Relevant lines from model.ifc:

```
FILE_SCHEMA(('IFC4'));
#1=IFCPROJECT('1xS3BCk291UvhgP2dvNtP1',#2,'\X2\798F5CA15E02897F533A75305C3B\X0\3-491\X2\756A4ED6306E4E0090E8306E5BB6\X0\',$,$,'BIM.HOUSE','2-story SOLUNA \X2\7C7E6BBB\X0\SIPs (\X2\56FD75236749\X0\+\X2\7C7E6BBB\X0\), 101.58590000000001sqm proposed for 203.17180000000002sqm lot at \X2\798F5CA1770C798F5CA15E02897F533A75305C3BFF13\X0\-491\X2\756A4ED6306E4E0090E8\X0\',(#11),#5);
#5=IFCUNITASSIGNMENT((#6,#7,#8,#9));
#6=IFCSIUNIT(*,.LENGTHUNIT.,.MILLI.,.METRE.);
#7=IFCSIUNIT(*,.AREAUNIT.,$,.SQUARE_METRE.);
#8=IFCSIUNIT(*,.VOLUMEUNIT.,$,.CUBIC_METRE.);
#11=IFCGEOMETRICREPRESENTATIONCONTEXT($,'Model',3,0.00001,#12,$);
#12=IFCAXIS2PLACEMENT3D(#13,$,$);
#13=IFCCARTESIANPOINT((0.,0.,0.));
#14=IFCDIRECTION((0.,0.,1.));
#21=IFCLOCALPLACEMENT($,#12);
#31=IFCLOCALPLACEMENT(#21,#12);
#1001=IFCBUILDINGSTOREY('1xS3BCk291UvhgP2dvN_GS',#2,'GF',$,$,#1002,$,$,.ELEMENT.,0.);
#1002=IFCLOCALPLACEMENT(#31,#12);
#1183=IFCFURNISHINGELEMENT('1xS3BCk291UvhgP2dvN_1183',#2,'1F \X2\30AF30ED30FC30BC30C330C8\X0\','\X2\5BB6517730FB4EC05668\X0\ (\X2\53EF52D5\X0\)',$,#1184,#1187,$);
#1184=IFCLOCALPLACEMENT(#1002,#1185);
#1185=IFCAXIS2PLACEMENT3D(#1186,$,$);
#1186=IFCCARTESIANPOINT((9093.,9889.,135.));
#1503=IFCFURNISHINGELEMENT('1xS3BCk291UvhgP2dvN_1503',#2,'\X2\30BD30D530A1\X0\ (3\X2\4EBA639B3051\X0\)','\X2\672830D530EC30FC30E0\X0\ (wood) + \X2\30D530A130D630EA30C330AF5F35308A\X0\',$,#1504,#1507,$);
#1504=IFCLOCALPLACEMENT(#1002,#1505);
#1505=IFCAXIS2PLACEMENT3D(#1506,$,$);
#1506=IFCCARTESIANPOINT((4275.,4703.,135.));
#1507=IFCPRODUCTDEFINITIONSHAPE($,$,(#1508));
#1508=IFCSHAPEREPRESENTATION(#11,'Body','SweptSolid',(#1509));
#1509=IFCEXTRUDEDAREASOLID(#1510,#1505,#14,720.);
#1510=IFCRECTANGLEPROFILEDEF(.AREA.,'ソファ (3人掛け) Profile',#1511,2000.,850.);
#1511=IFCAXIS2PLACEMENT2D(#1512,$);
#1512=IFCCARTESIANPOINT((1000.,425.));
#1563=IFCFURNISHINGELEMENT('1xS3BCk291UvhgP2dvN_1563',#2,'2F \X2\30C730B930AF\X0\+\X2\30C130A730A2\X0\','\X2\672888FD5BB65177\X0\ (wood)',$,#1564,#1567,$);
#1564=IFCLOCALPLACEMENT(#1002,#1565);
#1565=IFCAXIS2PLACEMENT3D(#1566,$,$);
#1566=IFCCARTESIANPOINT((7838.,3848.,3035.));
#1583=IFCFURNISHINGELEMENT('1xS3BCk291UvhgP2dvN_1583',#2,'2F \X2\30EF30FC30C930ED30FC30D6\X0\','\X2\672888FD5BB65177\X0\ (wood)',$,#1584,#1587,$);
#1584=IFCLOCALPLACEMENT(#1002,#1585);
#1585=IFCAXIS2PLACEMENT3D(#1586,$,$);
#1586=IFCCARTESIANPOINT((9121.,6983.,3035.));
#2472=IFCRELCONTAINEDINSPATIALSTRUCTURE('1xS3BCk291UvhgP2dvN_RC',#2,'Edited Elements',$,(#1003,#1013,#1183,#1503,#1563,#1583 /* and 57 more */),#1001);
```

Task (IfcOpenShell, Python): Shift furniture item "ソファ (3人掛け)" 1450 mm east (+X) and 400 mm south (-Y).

```python
import ifcopenshell
import ifcopenshell.api.geometry
import ifcopenshell.util.placement

model = ifcopenshell.open("model.ifc")

item = model.by_guid("1xS3BCk291UvhgP2dvN_1503")
matrix = ifcopenshell.util.placement.get_local_placement(item.ObjectPlacement)
matrix[0, 3] += 1450.0
matrix[1, 3] -= 400.0
ifcopenshell.api.geometry.edit_object_placement(model, product=item, matrix=matrix, is_si=False)

print(ifcopenshell.util.placement.get_local_placement(item.ObjectPlacement).round(3) + 0.0)

model.write("model_edited.ifc")
```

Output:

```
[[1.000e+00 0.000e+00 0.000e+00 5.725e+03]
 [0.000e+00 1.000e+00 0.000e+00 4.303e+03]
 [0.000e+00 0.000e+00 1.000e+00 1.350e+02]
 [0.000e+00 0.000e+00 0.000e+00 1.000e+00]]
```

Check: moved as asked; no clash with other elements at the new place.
